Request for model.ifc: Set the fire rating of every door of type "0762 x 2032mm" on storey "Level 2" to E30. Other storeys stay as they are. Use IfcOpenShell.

First a look at what the model holds.

```python
import ifcopenshell
import ifcopenshell.util.element

model = ifcopenshell.open("model.ifc")
print(model.schema)
storey = next(s for s in model.by_type("IfcBuildingStorey") if s.Name == "Level 2")
doors = [e for e in ifcopenshell.util.element.get_decomposition(storey) if e.is_a("IfcDoor")]
seen = {}
for e in doors:
    element_type = ifcopenshell.util.element.get_type(e)
    key = (element_type.Name if element_type != e and element_type else None, ifcopenshell.util.element.get_pset(e, "Pset_DoorCommon", "FireRating"))
    seen[key] = seen.get(key, 0) + 1
for (name, value), count in sorted(seen.items(), key=str):
    print(count, "x", name, "|", value)
```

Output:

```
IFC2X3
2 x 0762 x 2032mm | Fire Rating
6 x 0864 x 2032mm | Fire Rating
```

```python
import ifcopenshell
import ifcopenshell.api.pset
import ifcopenshell.util.element

model = ifcopenshell.open("model.ifc")

storey = next(s for s in model.by_type("IfcBuildingStorey") if s.Name == "Level 2")
doors = [e for e in ifcopenshell.util.element.get_decomposition(storey) if e.is_a("IfcDoor")]

count = 0
for e in doors:
    element_type = ifcopenshell.util.element.get_type(e)
    if element_type in (None, e) or element_type.Name != "0762 x 2032mm":
        continue
    # add_pset returns the element's existing set when there is one.
    pset = ifcopenshell.api.pset.add_pset(model, product=e, name="Pset_DoorCommon")
    ifcopenshell.api.pset.edit_pset(model, pset=pset, properties={"FireRating": "E30"})
    count += 1

print(count, "doors updated")

model.write("model_v2.ifc")
```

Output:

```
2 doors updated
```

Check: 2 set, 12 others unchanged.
